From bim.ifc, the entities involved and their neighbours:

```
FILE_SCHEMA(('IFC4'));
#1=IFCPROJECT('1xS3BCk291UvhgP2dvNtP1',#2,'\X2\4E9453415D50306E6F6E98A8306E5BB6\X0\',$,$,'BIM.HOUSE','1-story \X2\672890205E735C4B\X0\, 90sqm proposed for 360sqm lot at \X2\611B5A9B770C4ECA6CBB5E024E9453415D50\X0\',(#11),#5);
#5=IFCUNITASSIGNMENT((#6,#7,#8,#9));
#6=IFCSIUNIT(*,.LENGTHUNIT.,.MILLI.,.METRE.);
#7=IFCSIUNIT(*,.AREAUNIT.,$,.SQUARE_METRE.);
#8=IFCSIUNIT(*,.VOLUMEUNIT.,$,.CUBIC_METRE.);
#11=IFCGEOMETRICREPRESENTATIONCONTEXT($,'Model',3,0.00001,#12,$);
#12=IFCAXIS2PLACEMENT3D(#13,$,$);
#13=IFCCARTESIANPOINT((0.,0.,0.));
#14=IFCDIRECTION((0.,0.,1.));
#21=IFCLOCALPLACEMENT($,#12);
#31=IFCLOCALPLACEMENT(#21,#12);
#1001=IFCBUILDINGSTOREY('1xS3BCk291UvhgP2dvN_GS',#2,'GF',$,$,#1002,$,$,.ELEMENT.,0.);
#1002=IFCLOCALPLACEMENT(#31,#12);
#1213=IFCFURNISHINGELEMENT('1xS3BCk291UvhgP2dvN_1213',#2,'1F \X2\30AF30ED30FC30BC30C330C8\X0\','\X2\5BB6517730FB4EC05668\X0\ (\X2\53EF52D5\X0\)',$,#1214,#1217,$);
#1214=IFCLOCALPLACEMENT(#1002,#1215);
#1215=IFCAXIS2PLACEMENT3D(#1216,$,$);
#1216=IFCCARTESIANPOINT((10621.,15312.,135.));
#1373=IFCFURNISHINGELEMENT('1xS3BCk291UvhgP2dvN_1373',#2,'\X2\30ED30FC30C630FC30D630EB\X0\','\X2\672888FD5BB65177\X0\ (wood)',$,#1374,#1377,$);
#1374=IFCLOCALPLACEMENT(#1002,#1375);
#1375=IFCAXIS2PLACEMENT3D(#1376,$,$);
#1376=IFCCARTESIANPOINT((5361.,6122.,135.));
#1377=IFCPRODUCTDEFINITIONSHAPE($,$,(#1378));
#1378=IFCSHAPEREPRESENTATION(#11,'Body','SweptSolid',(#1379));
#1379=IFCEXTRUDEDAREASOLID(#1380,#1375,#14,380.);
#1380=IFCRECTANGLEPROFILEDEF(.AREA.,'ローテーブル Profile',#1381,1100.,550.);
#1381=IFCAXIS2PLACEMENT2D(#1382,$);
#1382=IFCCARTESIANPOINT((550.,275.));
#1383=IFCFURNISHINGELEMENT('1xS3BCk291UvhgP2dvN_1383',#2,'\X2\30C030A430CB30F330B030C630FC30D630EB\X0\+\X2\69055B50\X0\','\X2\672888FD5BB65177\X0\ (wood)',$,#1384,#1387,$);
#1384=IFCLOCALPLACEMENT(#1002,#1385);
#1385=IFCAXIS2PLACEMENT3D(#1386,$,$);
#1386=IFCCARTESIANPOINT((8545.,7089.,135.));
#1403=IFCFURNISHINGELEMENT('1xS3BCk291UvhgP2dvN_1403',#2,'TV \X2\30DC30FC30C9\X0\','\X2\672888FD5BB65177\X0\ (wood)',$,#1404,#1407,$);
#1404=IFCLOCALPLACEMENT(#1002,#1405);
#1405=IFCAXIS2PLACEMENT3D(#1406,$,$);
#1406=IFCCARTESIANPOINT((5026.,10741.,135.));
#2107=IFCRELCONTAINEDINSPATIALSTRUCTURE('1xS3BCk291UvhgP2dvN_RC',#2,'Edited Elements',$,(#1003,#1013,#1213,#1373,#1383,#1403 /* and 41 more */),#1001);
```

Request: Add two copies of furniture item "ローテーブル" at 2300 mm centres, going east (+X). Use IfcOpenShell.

```python
import numpy as np
import ifcopenshell
import ifcopenshell.api.geometry
import ifcopenshell.api.root
import ifcopenshell.util.element
import ifcopenshell.util.placement

model = ifcopenshell.open("bim.ifc")


def reuse_history(source, copy):
    """copy_class also copies each property set's owner history, people and application; keep the originals."""
    for rel in copy.IsDefinedBy:
        if rel.is_a("IfcRelDefinesByProperties") and (history := rel.RelatingPropertyDefinition.OwnerHistory):
            rel.RelatingPropertyDefinition.OwnerHistory = source.OwnerHistory
            ifcopenshell.util.element.remove_deep2(model, history)


source = model.by_guid("1xS3BCk291UvhgP2dvN_1373")
base = ifcopenshell.util.placement.get_local_placement(source.ObjectPlacement)
step = np.array([1.0, 0.0, 0.0]) * 2300.0

for i in range(1, 3):
    copy = ifcopenshell.api.root.copy_class(model, product=source)
    copy.Representation = ifcopenshell.util.element.copy_deep(
        model, source.Representation, exclude=["IfcGeometricRepresentationContext", "IfcRepresentationMap"]
    )
    reuse_history(source, copy)
    matrix = base.copy()
    matrix[:3, 3] += i * step
    print("added at", matrix[:3, 3].round(3) + 0.0)
    ifcopenshell.api.geometry.edit_object_placement(model, product=copy, matrix=matrix, is_si=False)

model.write("bim_edited.ifc")
```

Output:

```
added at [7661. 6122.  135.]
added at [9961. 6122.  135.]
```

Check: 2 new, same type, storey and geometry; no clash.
